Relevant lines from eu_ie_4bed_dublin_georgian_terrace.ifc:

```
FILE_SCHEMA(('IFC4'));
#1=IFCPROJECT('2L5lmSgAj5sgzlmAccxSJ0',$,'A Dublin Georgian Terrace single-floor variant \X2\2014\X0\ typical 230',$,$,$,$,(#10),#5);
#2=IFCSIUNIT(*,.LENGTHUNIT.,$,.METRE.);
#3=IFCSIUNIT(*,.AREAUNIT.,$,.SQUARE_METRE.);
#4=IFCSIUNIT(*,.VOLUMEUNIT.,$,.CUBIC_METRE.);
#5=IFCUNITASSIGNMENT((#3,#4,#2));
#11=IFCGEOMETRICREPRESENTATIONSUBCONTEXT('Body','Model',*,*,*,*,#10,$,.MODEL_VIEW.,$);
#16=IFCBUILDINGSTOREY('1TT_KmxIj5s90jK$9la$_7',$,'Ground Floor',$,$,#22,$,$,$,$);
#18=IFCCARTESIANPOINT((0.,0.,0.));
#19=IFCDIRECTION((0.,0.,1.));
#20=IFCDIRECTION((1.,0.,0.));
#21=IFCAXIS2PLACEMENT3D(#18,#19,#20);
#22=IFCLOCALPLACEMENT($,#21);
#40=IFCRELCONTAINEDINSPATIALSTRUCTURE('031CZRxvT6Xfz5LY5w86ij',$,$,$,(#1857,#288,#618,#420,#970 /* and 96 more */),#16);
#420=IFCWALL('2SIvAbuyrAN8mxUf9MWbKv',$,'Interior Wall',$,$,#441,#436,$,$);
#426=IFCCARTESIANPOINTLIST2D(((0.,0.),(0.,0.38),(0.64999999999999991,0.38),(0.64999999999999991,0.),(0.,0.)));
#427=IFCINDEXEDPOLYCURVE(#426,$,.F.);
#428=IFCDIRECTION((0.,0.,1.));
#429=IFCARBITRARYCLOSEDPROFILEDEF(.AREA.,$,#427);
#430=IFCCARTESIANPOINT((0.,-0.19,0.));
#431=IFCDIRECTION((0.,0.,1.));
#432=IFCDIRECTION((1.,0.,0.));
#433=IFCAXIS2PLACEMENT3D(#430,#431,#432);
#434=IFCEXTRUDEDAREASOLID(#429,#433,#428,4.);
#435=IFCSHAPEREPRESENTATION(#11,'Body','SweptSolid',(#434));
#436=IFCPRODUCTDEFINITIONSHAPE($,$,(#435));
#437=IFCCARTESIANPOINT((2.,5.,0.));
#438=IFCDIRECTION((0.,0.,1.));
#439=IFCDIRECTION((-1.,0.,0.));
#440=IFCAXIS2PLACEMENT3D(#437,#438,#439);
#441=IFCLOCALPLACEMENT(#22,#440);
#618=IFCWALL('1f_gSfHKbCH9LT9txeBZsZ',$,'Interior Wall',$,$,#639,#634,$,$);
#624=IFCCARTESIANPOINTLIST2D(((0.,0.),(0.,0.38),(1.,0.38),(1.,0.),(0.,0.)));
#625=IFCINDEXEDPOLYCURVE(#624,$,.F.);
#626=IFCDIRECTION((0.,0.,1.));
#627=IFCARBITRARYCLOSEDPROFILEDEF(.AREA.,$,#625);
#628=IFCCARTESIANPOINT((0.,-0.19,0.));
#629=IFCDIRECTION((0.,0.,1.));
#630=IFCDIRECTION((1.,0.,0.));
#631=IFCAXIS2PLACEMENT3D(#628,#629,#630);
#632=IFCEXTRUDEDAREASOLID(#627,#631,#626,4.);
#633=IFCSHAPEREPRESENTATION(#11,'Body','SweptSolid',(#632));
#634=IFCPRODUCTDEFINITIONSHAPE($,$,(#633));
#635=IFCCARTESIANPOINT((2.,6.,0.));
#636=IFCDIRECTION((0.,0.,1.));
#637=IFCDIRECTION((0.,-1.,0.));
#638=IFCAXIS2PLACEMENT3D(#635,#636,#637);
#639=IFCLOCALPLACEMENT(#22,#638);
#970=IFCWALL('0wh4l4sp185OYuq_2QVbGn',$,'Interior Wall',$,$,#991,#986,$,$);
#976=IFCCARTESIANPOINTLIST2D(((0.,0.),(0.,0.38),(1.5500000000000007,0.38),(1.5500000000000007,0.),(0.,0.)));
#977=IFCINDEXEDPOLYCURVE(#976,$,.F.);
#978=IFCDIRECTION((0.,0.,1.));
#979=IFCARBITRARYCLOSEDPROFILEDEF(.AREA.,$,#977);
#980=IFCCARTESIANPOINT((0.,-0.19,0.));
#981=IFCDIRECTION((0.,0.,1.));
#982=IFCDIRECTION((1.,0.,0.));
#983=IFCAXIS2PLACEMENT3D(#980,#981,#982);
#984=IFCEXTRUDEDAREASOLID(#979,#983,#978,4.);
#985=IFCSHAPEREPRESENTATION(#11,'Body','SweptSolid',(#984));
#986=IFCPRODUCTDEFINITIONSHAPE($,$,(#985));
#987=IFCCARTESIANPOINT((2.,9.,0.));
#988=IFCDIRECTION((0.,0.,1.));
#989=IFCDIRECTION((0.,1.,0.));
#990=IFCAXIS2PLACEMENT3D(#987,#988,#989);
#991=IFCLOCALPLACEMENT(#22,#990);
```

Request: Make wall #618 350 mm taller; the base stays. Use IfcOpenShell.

```python
import ifcopenshell
import ifcopenshell.geom
import ifcopenshell.util.representation
import ifcopenshell.util.shape
import ifcopenshell.util.unit

model = ifcopenshell.open("eu_ie_4bed_dublin_georgian_terrace.ifc")
unit_scale = ifcopenshell.util.unit.calculate_unit_scale(model)
settings = ifcopenshell.geom.settings()


def volume(element):
    """Net volume in cubic metres, openings subtracted."""
    shape = ifcopenshell.geom.create_shape(settings, element)
    return ifcopenshell.util.shape.get_volume(shape.geometry)


wall = model.by_id(618)
before = volume(wall)

body = ifcopenshell.util.representation.get_representation(wall, "Model", "Body")
solid = body.Items[0]
old_height = solid.Depth
solid.Depth += 0.35 / unit_scale
after = volume(wall)

print(f"height {old_height:g} -> {solid.Depth:g}, volume {before:.3f} -> {after:.3f} m3")

model.write("eu_ie_4bed_dublin_georgian_terrace_rev.ifc")
```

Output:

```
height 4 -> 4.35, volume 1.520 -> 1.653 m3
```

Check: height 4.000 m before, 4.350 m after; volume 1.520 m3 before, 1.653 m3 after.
